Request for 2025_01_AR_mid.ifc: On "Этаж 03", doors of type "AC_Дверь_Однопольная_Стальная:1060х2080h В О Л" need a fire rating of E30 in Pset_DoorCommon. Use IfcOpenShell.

First a look at what the model holds.

```python
import ifcopenshell
import ifcopenshell.util.element

model = ifcopenshell.open("2025_01_AR_mid.ifc")
print(model.schema)
storey = next(s for s in model.by_type("IfcBuildingStorey") if s.Name == "Этаж 03")
doors = [e for e in ifcopenshell.util.element.get_decomposition(storey) if e.is_a("IfcDoor")]
seen = {}
for e in doors:
    element_type = ifcopenshell.util.element.get_type(e)
    key = (element_type.Name if element_type != e and element_type else None, ifcopenshell.util.element.get_pset(e, "Pset_DoorCommon", "FireRating"))
    seen[key] = seen.get(key, 0) + 1
for (name, value), count in sorted(seen.items(), key=str):
    print(count, "x", name, "|", value)
```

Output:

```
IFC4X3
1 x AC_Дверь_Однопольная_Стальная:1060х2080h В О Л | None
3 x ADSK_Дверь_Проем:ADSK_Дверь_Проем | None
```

```python
import ifcopenshell
import ifcopenshell.api.pset
import ifcopenshell.util.element

model = ifcopenshell.open("2025_01_AR_mid.ifc")

storey = next(s for s in model.by_type("IfcBuildingStorey") if s.Name == "Этаж 03")
doors = [e for e in ifcopenshell.util.element.get_decomposition(storey) if e.is_a("IfcDoor")]

count = 0
for e in doors:
    element_type = ifcopenshell.util.element.get_type(e)
    if element_type in (None, e) or element_type.Name != "AC_Дверь_Однопольная_Стальная:1060х2080h В О Л":
        continue
    # add_pset returns the element's existing set when there is one.
    pset = ifcopenshell.api.pset.add_pset(model, product=e, name="Pset_DoorCommon")
    ifcopenshell.api.pset.edit_pset(model, pset=pset, properties={"FireRating": "E30"})
    count += 1

print(count, "doors updated")

model.write("2025_01_AR_mid_rev.ifc")
```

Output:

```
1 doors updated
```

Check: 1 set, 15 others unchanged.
